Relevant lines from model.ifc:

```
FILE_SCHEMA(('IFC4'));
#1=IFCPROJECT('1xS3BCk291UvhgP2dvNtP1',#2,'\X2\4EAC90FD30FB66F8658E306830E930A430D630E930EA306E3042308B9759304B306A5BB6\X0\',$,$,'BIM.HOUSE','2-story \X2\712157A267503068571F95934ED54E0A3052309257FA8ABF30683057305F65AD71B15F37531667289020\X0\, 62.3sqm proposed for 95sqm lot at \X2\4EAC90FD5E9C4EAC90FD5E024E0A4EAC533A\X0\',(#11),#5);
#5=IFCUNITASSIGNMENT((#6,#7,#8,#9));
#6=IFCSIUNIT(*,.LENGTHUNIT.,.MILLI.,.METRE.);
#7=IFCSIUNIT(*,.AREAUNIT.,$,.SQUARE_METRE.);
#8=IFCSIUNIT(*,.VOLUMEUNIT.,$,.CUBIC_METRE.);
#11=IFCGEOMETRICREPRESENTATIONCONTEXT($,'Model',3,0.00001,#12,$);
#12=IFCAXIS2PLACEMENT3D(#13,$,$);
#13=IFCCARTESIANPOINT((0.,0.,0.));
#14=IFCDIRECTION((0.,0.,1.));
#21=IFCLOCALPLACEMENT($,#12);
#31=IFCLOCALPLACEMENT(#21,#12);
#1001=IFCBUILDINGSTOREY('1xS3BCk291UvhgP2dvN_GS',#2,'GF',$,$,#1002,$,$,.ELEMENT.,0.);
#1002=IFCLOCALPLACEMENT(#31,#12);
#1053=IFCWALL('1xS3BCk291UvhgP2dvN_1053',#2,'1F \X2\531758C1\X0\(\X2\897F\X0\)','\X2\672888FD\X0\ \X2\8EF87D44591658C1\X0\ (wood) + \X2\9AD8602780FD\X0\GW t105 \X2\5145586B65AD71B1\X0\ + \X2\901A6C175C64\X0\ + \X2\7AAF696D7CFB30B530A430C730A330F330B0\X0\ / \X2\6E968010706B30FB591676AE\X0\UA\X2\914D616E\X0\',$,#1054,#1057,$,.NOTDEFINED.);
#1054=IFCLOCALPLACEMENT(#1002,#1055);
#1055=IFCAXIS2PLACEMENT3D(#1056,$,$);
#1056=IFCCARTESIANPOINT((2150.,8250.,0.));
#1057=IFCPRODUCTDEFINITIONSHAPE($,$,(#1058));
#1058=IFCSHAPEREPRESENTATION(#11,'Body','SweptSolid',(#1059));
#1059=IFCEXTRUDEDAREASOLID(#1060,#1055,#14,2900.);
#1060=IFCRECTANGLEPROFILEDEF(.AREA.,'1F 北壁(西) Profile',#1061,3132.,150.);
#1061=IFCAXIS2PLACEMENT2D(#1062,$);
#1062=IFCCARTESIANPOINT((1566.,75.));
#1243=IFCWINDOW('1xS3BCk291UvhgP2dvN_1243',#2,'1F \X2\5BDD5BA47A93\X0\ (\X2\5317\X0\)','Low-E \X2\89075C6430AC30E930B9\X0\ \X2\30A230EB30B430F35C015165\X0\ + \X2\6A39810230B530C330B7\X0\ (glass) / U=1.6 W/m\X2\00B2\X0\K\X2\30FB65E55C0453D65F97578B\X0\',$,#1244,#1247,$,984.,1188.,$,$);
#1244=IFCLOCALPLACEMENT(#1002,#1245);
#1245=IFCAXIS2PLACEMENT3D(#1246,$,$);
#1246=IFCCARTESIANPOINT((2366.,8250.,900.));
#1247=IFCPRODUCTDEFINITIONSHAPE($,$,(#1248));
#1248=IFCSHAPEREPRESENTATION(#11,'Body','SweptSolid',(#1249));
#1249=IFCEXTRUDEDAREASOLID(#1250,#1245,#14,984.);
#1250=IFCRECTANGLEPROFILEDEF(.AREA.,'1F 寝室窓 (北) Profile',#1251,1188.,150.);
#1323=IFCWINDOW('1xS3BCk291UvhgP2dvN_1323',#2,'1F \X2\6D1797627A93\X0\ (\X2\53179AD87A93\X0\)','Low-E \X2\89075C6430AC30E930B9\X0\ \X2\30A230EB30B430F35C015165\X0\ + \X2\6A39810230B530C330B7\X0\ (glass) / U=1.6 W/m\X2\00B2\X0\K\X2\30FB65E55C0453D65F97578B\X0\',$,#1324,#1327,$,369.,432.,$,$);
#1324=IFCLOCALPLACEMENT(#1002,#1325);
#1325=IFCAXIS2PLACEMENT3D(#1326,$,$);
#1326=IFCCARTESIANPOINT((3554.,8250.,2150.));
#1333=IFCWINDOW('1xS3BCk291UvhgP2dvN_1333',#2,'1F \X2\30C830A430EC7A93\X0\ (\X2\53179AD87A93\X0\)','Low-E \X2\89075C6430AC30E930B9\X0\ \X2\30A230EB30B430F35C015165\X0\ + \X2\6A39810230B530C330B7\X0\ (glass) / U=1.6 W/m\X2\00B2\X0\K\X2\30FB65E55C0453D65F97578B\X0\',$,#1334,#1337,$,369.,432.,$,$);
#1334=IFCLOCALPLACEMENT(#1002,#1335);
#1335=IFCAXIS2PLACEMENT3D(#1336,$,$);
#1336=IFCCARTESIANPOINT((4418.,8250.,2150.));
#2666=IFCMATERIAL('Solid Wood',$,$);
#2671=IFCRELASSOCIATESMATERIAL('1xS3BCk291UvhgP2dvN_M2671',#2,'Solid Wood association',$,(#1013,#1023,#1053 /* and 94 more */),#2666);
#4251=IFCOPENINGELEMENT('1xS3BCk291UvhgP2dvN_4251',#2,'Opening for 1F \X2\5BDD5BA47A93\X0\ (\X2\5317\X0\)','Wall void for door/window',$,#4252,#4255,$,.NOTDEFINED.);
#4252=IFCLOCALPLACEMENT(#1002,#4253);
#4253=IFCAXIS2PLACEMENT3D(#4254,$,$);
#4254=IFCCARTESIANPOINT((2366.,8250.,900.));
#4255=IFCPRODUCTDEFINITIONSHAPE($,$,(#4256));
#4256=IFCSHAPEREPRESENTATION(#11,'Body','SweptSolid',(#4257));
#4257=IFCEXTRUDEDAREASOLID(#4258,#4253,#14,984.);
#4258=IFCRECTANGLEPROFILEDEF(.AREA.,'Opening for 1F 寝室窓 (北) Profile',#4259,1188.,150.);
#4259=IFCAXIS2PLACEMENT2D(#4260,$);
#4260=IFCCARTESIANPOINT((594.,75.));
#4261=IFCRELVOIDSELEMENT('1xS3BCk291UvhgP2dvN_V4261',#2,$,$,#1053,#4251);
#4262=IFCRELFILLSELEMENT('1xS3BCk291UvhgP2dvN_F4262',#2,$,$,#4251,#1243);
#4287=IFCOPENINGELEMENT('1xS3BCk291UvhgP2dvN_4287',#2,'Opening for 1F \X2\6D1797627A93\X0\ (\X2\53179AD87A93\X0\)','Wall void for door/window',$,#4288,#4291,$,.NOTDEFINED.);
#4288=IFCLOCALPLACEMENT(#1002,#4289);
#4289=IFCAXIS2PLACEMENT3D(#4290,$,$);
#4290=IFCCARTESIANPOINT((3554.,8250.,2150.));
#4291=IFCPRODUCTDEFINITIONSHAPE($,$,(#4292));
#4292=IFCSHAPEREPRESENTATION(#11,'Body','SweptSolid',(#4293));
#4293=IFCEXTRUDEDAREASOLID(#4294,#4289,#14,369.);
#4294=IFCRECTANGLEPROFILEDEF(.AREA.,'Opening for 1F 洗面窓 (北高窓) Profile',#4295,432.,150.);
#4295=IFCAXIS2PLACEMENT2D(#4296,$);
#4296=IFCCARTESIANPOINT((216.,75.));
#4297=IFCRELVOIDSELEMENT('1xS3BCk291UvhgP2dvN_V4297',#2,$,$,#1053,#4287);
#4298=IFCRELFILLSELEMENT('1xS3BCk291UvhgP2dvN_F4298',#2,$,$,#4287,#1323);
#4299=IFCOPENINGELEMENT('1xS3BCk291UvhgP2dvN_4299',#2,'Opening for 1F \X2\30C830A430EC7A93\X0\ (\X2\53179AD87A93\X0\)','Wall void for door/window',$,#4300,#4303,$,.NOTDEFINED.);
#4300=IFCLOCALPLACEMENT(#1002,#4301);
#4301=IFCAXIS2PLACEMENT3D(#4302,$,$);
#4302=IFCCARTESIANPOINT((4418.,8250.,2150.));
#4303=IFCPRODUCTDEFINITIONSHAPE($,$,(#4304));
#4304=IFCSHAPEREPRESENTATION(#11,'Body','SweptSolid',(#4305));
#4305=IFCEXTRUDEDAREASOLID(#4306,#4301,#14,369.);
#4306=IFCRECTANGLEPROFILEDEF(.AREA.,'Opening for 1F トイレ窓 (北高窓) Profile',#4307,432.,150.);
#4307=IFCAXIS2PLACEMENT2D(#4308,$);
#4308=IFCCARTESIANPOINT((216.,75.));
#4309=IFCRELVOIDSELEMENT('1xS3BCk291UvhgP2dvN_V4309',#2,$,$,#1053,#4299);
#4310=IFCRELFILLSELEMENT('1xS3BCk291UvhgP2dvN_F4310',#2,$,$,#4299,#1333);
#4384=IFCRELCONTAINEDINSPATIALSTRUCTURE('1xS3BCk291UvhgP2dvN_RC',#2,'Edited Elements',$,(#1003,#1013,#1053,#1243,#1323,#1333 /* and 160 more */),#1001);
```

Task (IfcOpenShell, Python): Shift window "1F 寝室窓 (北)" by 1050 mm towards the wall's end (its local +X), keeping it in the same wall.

```python
import ifcopenshell
import ifcopenshell.api.geometry
import ifcopenshell.util.placement
import ifcopenshell.util.unit

model = ifcopenshell.open("model.ifc")
unit_scale = ifcopenshell.util.unit.calculate_unit_scale(model)

window = model.by_id(1243)
opening = window.FillsVoids[0].RelatingOpeningElement
wall = opening.VoidsElements[0].RelatingBuildingElement

wall_matrix = ifcopenshell.util.placement.get_local_placement(wall.ObjectPlacement)
shift = wall_matrix[:3, 0] * 1.05 / unit_scale
before = ifcopenshell.util.placement.get_local_placement(window.ObjectPlacement)[:3, 3].copy()

# The window is not placed relative to its opening, so move both.
for product in (opening, window):
    matrix = ifcopenshell.util.placement.get_local_placement(product.ObjectPlacement)
    matrix[:3, 3] += shift
    ifcopenshell.api.geometry.edit_object_placement(model, product=product, matrix=matrix, is_si=False)

after = ifcopenshell.util.placement.get_local_placement(window.ObjectPlacement)[:3, 3]
print("window moved by", (after - before).round(3) + 0.0)

model.write("model-out.ifc")
```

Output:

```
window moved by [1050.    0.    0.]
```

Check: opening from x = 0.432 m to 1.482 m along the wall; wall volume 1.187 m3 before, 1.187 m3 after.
